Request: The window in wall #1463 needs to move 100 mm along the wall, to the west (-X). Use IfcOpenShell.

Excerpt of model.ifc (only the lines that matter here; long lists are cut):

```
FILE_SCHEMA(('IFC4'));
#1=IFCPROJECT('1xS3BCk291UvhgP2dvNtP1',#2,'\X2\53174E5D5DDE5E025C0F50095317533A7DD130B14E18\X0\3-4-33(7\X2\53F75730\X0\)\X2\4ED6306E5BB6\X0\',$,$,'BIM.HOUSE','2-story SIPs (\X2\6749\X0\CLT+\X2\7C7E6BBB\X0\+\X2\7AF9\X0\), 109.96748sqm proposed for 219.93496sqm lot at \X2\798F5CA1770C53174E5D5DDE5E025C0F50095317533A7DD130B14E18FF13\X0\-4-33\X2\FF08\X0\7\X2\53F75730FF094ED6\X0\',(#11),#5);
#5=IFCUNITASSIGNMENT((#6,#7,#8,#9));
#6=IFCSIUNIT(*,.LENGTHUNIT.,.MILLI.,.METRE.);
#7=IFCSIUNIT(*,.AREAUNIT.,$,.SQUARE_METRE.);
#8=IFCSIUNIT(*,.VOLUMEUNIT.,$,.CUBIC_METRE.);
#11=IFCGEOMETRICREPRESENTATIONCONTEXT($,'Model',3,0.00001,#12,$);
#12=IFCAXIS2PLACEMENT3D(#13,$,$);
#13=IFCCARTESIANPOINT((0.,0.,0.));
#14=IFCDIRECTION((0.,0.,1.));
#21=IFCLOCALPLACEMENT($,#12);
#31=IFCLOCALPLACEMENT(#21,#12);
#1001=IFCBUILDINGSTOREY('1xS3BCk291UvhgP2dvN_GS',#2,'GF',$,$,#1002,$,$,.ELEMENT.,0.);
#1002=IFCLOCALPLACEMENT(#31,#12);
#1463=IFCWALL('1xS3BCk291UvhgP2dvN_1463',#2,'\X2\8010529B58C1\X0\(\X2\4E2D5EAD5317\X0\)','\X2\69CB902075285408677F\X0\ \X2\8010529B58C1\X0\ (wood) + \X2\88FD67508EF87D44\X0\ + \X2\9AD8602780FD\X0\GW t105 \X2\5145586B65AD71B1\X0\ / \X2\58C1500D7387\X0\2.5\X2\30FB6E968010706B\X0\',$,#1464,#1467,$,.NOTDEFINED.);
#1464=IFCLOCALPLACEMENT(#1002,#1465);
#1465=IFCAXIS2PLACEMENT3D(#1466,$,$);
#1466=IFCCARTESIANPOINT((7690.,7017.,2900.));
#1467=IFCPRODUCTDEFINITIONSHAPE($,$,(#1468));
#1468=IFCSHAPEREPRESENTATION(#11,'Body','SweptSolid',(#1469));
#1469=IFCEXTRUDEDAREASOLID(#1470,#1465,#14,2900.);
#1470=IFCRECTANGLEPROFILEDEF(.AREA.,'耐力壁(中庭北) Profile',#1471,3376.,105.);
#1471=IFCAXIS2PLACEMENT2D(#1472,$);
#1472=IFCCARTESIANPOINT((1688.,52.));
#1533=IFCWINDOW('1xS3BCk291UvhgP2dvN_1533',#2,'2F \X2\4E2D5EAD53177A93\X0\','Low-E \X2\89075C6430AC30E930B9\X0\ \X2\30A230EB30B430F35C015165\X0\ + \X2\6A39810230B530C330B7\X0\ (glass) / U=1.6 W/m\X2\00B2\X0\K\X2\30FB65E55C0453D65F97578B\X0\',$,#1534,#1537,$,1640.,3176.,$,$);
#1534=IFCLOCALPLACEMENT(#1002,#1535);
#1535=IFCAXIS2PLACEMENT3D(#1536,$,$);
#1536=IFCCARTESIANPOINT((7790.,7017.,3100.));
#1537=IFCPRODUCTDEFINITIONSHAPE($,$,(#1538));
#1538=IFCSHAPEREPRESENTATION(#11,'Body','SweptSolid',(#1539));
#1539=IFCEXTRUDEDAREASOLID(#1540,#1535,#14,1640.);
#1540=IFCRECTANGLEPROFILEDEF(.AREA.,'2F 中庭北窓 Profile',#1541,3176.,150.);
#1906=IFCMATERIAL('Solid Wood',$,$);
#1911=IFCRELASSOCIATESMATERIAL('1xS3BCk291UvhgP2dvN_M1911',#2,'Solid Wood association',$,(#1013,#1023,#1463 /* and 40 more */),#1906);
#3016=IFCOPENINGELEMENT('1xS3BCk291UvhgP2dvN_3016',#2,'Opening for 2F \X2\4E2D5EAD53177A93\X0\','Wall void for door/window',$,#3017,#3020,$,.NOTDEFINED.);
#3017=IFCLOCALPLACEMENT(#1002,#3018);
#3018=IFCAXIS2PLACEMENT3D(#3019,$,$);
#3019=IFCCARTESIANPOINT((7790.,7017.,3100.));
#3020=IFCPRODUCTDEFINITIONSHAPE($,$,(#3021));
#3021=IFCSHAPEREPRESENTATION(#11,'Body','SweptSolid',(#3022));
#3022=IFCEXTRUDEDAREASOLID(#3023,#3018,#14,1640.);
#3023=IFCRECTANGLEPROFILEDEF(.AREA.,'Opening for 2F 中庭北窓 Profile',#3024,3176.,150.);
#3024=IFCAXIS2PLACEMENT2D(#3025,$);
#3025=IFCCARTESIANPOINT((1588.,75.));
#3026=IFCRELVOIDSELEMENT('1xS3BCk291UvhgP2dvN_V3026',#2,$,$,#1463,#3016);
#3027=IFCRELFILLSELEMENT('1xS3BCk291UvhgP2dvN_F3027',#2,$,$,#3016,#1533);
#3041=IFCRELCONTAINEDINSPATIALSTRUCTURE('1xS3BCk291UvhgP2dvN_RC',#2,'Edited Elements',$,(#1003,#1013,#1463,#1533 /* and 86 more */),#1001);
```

```python
import ifcopenshell
import ifcopenshell.api.geometry
import ifcopenshell.util.placement

model = ifcopenshell.open("model.ifc")

window = model.by_guid("1xS3BCk291UvhgP2dvN_1533")
opening = window.FillsVoids[0].RelatingOpeningElement
wall = opening.VoidsElements[0].RelatingBuildingElement

wall_matrix = ifcopenshell.util.placement.get_local_placement(wall.ObjectPlacement)
shift = wall_matrix[:3, 0] * -100.0
before = ifcopenshell.util.placement.get_local_placement(window.ObjectPlacement)[:3, 3].copy()

# The window is not placed relative to its opening, so move both.
for product in (opening, window):
    matrix = ifcopenshell.util.placement.get_local_placement(product.ObjectPlacement)
    matrix[:3, 3] += shift
    ifcopenshell.api.geometry.edit_object_placement(model, product=product, matrix=matrix, is_si=False)

after = ifcopenshell.util.placement.get_local_placement(window.ObjectPlacement)[:3, 3]
print("window moved by", (after - before).round(3) + 0.0)

model.write("model-out.ifc")
```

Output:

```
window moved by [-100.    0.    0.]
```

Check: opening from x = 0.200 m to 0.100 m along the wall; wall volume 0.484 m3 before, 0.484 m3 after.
